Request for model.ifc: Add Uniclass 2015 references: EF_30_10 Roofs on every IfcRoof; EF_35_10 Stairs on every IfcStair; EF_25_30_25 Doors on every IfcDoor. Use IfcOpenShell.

First a look at what the model holds.

```python
import ifcopenshell

model = ifcopenshell.open("model.ifc")
print(model.schema)
print("classifications:", [c.Name for c in model.by_type("IfcClassification")])
for ifc_class in ("IfcDoor", "IfcRoof", "IfcStair", "IfcWall", "IfcWindow"):
    print(ifc_class, len(model.by_type(ifc_class)))
```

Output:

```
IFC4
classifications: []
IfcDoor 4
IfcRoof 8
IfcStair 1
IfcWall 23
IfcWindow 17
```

```python
import ifcopenshell
import ifcopenshell.api.classification

model = ifcopenshell.open("model.ifc")

system = ifcopenshell.api.classification.add_classification(model, classification="Uniclass 2015")

codes = {
    "IfcRoof": ("EF_30_10", "Roofs"),
    "IfcStair": ("EF_35_10", "Stairs"),
    "IfcDoor": ("EF_25_30_25", "Doors"),
}
for ifc_class, (code, name) in codes.items():
    products = model.by_type(ifc_class)
    ifcopenshell.api.classification.add_reference(
        model, products=products, classification=system, identification=code, name=name
    )
    print(code, len(products))

model.write("model_v2.ifc")
```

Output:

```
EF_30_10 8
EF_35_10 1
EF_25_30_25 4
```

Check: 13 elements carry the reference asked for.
